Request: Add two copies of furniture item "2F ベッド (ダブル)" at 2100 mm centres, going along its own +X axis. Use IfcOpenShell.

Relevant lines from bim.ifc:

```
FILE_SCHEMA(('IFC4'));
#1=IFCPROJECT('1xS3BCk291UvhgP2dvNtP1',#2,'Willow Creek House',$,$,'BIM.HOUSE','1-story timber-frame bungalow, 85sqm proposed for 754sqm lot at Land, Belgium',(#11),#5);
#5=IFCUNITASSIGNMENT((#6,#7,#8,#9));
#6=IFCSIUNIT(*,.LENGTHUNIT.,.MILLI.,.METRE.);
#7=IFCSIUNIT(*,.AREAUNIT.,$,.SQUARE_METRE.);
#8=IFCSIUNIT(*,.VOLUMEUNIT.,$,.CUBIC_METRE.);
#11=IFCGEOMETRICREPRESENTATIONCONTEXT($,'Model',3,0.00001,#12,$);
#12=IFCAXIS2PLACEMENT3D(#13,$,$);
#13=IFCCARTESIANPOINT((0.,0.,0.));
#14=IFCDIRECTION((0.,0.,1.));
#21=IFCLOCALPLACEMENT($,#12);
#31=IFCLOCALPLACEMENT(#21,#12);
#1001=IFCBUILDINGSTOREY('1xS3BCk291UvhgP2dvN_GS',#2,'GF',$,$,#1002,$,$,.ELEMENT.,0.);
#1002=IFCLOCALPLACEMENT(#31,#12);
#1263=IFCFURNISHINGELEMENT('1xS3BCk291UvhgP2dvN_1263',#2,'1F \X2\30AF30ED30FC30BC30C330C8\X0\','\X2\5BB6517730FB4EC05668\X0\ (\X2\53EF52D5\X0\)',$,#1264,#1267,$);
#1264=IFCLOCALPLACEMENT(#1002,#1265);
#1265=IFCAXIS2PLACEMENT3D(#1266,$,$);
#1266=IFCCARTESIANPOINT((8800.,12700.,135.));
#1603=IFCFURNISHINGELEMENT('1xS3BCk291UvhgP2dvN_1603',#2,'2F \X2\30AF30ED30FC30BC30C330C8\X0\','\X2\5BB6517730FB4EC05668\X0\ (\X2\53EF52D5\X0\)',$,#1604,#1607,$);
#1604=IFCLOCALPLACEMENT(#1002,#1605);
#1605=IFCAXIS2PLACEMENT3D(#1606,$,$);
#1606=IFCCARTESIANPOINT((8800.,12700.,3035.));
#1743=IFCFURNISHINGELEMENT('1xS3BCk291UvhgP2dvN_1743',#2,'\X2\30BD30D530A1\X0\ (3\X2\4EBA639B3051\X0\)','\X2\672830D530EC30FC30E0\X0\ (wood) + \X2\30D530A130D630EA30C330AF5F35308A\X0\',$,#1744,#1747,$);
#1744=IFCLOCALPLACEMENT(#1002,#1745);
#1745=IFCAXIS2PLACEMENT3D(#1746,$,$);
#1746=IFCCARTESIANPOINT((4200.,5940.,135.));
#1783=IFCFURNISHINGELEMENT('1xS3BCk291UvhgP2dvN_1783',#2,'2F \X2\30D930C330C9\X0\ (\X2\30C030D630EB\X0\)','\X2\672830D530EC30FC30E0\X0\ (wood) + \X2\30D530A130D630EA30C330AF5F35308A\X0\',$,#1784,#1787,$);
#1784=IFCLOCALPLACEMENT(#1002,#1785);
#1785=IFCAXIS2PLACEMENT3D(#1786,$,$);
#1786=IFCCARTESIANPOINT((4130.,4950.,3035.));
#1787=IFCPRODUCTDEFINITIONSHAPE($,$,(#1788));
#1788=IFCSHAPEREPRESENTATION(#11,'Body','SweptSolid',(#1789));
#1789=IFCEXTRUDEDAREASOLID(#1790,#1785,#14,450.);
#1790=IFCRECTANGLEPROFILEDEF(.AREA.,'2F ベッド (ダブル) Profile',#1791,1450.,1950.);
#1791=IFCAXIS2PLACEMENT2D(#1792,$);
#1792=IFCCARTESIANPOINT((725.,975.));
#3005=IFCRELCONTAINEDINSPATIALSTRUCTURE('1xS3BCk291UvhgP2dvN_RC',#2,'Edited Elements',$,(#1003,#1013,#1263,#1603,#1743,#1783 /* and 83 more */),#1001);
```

```python
import ifcopenshell
import ifcopenshell.api.geometry
import ifcopenshell.api.root
import ifcopenshell.util.element
import ifcopenshell.util.placement

model = ifcopenshell.open("bim.ifc")


def reuse_history(source, copy):
    """copy_class also copies each property set's owner history, people and application; keep the originals."""
    for rel in copy.IsDefinedBy:
        if rel.is_a("IfcRelDefinesByProperties") and (history := rel.RelatingPropertyDefinition.OwnerHistory):
            rel.RelatingPropertyDefinition.OwnerHistory = source.OwnerHistory
            ifcopenshell.util.element.remove_deep2(model, history)


source = model.by_guid("1xS3BCk291UvhgP2dvN_1783")
base = ifcopenshell.util.placement.get_local_placement(source.ObjectPlacement)
step = base[:3, 0] * 2100.0

for i in range(1, 3):
    copy = ifcopenshell.api.root.copy_class(model, product=source)
    copy.Representation = ifcopenshell.util.element.copy_deep(
        model, source.Representation, exclude=["IfcGeometricRepresentationContext", "IfcRepresentationMap"]
    )
    reuse_history(source, copy)
    matrix = base.copy()
    matrix[:3, 3] += i * step
    print("added at", matrix[:3, 3].round(3) + 0.0)
    ifcopenshell.api.geometry.edit_object_placement(model, product=copy, matrix=matrix, is_si=False)

model.write("bim_rev.ifc")
```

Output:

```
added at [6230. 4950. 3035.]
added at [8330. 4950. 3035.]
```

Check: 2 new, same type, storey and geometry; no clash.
